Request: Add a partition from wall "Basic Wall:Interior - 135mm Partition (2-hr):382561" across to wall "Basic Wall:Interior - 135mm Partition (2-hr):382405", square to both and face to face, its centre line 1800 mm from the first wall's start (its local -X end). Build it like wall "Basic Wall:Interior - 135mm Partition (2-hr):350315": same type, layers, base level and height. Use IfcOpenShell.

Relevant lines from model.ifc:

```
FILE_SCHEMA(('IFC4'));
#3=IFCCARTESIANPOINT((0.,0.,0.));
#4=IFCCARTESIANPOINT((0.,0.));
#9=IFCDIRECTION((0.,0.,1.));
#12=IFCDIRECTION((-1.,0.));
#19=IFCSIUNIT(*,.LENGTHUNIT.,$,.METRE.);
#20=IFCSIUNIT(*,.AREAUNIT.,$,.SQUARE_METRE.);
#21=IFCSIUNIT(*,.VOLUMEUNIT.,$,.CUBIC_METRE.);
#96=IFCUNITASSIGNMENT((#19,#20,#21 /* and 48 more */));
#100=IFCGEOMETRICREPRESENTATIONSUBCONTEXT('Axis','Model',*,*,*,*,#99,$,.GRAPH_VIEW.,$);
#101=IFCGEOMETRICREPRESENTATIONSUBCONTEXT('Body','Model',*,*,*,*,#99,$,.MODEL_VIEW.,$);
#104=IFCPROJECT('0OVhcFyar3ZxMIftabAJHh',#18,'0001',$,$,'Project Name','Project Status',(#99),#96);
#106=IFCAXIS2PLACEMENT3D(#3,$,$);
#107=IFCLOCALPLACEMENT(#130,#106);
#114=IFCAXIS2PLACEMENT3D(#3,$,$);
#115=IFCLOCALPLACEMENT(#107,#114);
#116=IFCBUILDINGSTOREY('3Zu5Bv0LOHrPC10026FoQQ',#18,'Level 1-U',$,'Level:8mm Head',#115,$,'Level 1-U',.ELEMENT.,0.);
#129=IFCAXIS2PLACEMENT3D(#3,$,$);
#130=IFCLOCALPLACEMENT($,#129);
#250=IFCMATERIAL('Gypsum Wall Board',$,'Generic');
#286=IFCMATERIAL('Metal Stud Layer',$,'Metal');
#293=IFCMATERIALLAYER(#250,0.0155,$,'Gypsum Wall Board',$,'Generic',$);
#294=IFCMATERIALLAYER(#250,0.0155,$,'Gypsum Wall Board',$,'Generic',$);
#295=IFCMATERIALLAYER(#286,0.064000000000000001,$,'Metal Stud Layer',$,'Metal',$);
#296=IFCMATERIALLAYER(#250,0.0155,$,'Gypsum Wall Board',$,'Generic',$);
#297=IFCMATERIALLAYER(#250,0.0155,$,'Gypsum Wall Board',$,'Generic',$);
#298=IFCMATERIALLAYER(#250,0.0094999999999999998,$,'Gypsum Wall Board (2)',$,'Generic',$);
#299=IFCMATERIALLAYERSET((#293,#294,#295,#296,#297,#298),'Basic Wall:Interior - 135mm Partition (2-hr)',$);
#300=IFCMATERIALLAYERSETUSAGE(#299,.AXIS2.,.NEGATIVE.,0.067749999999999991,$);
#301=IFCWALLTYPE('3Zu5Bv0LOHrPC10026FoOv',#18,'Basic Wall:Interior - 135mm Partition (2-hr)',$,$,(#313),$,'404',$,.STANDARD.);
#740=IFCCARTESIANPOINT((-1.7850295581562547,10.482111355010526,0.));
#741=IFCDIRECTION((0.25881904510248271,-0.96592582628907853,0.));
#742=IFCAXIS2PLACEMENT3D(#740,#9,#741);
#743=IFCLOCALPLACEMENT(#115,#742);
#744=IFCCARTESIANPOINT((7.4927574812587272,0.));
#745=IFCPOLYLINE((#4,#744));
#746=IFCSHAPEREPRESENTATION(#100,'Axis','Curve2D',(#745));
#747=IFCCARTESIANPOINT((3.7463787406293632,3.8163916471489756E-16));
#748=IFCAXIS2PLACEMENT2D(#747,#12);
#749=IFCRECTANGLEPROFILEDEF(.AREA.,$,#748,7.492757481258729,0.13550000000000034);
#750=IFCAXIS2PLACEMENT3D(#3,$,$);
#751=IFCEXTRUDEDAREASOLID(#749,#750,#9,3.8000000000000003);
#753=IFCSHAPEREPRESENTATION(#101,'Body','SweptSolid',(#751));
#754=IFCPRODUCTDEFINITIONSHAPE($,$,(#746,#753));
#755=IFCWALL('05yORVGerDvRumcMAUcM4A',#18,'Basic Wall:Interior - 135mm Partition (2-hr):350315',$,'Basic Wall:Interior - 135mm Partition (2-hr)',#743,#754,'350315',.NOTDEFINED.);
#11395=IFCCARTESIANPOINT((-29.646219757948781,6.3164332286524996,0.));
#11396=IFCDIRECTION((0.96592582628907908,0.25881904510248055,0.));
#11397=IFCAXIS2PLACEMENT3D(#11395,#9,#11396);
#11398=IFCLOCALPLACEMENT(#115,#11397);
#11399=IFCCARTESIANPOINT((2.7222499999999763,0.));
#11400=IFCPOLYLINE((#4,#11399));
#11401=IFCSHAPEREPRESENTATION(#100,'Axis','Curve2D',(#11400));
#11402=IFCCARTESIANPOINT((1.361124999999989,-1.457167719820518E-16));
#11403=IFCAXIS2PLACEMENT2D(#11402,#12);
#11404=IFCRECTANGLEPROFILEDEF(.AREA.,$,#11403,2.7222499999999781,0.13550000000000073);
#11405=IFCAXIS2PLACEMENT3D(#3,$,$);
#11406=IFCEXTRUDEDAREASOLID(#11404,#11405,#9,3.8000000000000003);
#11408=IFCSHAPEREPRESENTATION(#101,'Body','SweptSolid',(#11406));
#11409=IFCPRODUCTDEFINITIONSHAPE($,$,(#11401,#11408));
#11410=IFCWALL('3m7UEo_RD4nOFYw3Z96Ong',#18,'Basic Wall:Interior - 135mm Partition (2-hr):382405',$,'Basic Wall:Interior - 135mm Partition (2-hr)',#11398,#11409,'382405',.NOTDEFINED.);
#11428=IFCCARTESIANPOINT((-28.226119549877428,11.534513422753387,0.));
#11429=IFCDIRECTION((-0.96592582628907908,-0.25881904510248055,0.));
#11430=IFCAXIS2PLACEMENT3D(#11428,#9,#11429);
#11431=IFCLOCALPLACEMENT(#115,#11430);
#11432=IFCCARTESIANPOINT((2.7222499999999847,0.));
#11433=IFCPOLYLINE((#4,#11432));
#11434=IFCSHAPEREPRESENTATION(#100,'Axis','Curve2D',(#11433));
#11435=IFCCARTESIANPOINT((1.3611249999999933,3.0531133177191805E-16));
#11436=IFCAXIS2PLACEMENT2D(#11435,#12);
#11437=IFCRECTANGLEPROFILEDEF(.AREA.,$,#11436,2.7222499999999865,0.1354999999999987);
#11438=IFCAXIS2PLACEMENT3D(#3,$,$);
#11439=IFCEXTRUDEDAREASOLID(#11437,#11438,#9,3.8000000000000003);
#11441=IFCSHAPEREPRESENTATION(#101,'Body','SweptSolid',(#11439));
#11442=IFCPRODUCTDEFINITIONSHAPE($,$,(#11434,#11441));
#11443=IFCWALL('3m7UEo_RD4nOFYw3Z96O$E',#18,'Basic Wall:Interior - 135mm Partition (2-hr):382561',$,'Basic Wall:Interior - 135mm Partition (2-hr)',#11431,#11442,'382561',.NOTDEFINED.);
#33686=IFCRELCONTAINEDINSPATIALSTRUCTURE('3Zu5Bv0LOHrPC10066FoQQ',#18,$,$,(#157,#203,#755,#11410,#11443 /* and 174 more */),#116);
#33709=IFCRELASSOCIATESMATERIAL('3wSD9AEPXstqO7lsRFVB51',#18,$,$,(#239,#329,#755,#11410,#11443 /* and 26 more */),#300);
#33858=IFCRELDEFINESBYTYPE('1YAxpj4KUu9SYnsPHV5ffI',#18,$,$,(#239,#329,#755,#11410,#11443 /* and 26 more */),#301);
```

```python
import numpy as np
import ifcopenshell
import ifcopenshell.api.geometry
import ifcopenshell.api.material
import ifcopenshell.api.pset
import ifcopenshell.api.root
import ifcopenshell.api.spatial
import ifcopenshell.api.type
import ifcopenshell.geom
import ifcopenshell.util.element
import ifcopenshell.util.placement
import ifcopenshell.util.representation
import ifcopenshell.util.shape
import ifcopenshell.util.unit

model = ifcopenshell.open("model.ifc")
unit_scale = ifcopenshell.util.unit.calculate_unit_scale(model)
settings = ifcopenshell.geom.settings()
settings.set("use-world-coords", True)

start_wall = model.by_id(11443)
end_wall = model.by_guid("3m7UEo_RD4nOFYw3Z96Ong")
like = model.by_guid("05yORVGerDvRumcMAUcM4A")
matrix = ifcopenshell.util.placement.get_local_placement(start_wall.ObjectPlacement)
matrix[:3, 3] *= unit_scale


def extent(element):
    """Bounding box in the first wall's axes, in metres."""
    shape = ifcopenshell.geom.create_shape(settings, element)
    points = (ifcopenshell.util.shape.get_vertices(shape.geometry) - matrix[:3, 3]) @ matrix[:3, :3]
    return points.min(axis=0), points.max(axis=0)


y_start = extent(start_wall)[1][1]
y_end = extent(end_wall)[0][1]
like_min, like_max = extent(like)
length, height = float(abs(y_end - y_start)), float(like_max[2] - like_min[2])
layer_set = ifcopenshell.util.element.get_material(like, should_skip_usage=True)
thickness = sum(layer.LayerThickness for layer in layer_set.MaterialLayers) * unit_scale

wall = ifcopenshell.api.root.create_entity(model, ifc_class="IfcWall", name="New partition")
storey = ifcopenshell.util.element.get_container(like)
ifcopenshell.api.spatial.assign_container(model, products=[wall], relating_structure=storey)
ifcopenshell.api.type.assign_type(
    model, related_objects=[wall], relating_type=ifcopenshell.util.element.get_type(like), should_map_representations=False
)
rel = ifcopenshell.api.material.assign_material(
    model, products=[wall], type="IfcMaterialLayerSetUsage", material=layer_set
)
rel.RelatingMaterial.OffsetFromReferenceLine = -thickness / 2 / unit_scale
pset = ifcopenshell.api.pset.add_pset(model, product=wall, name="Pset_WallCommon")
ifcopenshell.api.pset.edit_pset(model, pset=pset, properties={"IsExternal": False, "LoadBearing": False})

# The axis runs down the middle of the wall.
axis = ifcopenshell.api.geometry.add_axis_representation(
    model, context=ifcopenshell.util.representation.get_context(model, "Model", "Axis"), axis=[(0.0, 0.0), (length, 0.0)]
)
body = ifcopenshell.api.geometry.add_wall_representation(
    model,
    context=ifcopenshell.util.representation.get_context(model, "Model", "Body", "MODEL_VIEW"),
    length=length,
    height=height,
    thickness=thickness,
    offset=-thickness / 2,
)
for representation in (axis, body):
    ifcopenshell.api.geometry.assign_representation(model, product=wall, representation=representation)

placement = matrix @ ifcopenshell.util.placement.rotation(90, "Z")
placement[:, 3] = matrix @ np.array([extent(start_wall)[0][0] + 1.8, y_start, like_min[2], 1.0])
ifcopenshell.api.geometry.edit_object_placement(model, product=wall, matrix=placement)

print(f"partition {length:.3f} m long, {height:.3f} m high, {thickness:.3f} m thick")

model.write("model_edited.ifc")
```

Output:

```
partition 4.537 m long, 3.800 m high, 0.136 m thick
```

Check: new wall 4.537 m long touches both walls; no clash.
